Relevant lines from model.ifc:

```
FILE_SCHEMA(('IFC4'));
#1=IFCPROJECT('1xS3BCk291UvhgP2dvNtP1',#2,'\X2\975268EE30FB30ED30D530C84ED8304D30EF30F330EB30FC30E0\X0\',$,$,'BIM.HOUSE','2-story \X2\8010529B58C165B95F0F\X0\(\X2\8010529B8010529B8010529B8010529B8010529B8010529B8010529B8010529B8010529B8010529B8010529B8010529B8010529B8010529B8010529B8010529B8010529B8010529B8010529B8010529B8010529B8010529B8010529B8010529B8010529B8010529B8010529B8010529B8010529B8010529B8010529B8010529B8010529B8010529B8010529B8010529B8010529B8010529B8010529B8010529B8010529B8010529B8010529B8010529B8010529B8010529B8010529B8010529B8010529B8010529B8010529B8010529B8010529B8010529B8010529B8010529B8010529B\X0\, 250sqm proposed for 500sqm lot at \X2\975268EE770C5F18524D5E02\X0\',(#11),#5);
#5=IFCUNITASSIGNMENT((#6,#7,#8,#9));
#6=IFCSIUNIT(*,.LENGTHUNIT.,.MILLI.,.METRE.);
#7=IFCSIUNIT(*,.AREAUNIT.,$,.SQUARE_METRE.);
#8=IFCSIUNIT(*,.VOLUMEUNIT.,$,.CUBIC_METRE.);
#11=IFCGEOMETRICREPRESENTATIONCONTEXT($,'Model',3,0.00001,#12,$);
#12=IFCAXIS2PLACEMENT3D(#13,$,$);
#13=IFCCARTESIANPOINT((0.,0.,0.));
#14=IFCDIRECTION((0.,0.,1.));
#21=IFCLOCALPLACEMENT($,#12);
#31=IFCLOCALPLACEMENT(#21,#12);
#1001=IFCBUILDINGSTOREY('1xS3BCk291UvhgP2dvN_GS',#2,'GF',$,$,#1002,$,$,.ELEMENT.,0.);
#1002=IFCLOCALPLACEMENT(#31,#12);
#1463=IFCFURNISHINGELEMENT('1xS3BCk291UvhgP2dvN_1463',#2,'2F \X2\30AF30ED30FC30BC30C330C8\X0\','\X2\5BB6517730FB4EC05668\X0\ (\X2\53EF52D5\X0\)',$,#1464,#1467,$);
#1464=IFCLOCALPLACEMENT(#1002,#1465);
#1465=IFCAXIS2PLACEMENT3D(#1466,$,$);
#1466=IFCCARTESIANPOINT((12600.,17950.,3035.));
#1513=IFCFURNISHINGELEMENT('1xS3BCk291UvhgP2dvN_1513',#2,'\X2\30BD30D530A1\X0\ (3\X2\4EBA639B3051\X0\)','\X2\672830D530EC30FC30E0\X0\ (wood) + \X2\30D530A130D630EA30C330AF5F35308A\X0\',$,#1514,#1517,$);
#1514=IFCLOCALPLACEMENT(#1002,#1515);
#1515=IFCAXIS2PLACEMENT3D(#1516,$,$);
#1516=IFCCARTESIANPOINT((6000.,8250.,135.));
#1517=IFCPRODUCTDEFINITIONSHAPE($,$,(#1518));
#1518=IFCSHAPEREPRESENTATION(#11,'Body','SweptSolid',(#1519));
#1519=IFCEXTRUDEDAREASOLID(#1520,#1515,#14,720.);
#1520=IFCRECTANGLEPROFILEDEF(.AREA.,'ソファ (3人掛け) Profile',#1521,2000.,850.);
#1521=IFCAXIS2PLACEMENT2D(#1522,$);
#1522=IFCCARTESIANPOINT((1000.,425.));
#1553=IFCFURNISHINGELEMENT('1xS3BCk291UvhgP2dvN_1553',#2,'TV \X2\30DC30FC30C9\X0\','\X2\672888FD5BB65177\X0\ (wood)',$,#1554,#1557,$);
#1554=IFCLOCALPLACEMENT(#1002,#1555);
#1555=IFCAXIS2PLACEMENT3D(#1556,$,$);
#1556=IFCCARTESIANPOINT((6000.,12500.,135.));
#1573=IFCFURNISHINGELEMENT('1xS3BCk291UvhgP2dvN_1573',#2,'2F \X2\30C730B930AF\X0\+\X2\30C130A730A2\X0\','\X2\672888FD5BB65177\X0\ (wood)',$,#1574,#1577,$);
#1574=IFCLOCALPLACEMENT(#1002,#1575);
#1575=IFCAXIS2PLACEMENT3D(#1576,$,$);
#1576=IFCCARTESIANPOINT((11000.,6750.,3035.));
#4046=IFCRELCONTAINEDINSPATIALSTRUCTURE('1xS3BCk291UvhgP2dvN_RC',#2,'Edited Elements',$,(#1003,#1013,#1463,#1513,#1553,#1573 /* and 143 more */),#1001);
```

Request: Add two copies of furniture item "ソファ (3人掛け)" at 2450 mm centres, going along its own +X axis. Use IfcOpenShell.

```python
import ifcopenshell
import ifcopenshell.api.geometry
import ifcopenshell.api.root
import ifcopenshell.util.element
import ifcopenshell.util.placement

model = ifcopenshell.open("model.ifc")


def reuse_history(source, copy):
    """copy_class also copies each property set's owner history, people and application; keep the originals."""
    for rel in copy.IsDefinedBy:
        if rel.is_a("IfcRelDefinesByProperties") and (history := rel.RelatingPropertyDefinition.OwnerHistory):
            rel.RelatingPropertyDefinition.OwnerHistory = source.OwnerHistory
            ifcopenshell.util.element.remove_deep2(model, history)


source = model.by_guid("1xS3BCk291UvhgP2dvN_1513")
base = ifcopenshell.util.placement.get_local_placement(source.ObjectPlacement)
step = base[:3, 0] * 2450.0

for i in range(1, 3):
    copy = ifcopenshell.api.root.copy_class(model, product=source)
    copy.Representation = ifcopenshell.util.element.copy_deep(
        model, source.Representation, exclude=["IfcGeometricRepresentationContext", "IfcRepresentationMap"]
    )
    reuse_history(source, copy)
    matrix = base.copy()
    matrix[:3, 3] += i * step
    print("added at", matrix[:3, 3].round(3) + 0.0)
    ifcopenshell.api.geometry.edit_object_placement(model, product=copy, matrix=matrix, is_si=False)

model.write("model_rev.ifc")
```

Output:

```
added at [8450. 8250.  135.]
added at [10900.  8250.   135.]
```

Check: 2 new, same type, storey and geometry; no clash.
